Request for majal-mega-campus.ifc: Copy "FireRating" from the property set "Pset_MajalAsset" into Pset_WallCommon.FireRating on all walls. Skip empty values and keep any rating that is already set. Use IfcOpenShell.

First a look at what the model holds.

```python
import ifcopenshell
import ifcopenshell.util.element

model = ifcopenshell.open("majal-mega-campus.ifc")
print(model.schema)
walls = model.by_type("IfcWall")
print(len(walls), "walls")
for e in walls[:8]:
    source = ifcopenshell.util.element.get_pset(e, "Pset_MajalAsset", "FireRating")
    target = ifcopenshell.util.element.get_pset(e, "Pset_WallCommon", "FireRating")
    print(e.id(), repr(source), repr(target), sep=" | ")
```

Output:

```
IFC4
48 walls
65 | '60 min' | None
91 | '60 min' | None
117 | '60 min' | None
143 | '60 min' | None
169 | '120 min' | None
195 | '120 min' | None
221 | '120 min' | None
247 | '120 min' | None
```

```python
import ifcopenshell
import ifcopenshell.api.pset
import ifcopenshell.util.element

model = ifcopenshell.open("majal-mega-campus.ifc")

count = 0
for e in model.by_type("IfcWall"):
    value = ifcopenshell.util.element.get_pset(e, "Pset_MajalAsset", "FireRating")
    current = ifcopenshell.util.element.get_pset(e, "Pset_WallCommon", "FireRating")
    if not value or not value.strip() or current:
        continue
    # add_pset returns the element's existing set when there is one.
    pset = ifcopenshell.api.pset.add_pset(model, product=e, name="Pset_WallCommon")
    ifcopenshell.api.pset.edit_pset(model, pset=pset, properties={"FireRating": value})
    count += 1

print(count, "walls updated")

model.write("majal-mega-campus-out.ifc")
```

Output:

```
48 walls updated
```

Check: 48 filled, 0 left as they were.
